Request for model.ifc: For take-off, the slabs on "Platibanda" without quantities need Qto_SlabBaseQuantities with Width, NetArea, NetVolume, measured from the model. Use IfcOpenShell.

First a look at what the model holds.

```python
import ifcopenshell
import ifcopenshell.util.element
import ifcopenshell.util.unit

model = ifcopenshell.open("model.ifc")
print(model.schema)
for unit_type in ("LENGTHUNIT", "AREAUNIT", "VOLUMEUNIT"):
    print(unit_type, ifcopenshell.util.unit.calculate_unit_scale(model, unit_type))
storey = next(s for s in model.by_type("IfcBuildingStorey") if s.Name == "Platibanda")
slabs = [e for e in ifcopenshell.util.element.get_decomposition(storey) if e.is_a("IfcSlab")]
for e in sorted(slabs, key=lambda e: e.id()):
    print(e.id(), e.is_a(), e.Name, list(ifcopenshell.util.element.get_psets(e, qtos_only=True)), sep=" | ")
```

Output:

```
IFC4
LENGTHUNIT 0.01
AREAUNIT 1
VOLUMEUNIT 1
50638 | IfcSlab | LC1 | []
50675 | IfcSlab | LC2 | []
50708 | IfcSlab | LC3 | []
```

```python
import ifcopenshell
import ifcopenshell.api.pset
import ifcopenshell.geom
import ifcopenshell.util.element
import ifcopenshell.util.shape
import ifcopenshell.util.unit

model = ifcopenshell.open("model.ifc")
unit_scale = ifcopenshell.util.unit.calculate_unit_scale(model)
area_scale = ifcopenshell.util.unit.calculate_unit_scale(model, "AREAUNIT")
volume_scale = ifcopenshell.util.unit.calculate_unit_scale(model, "VOLUMEUNIT")
settings = ifcopenshell.geom.settings()

storey = next(s for s in model.by_type("IfcBuildingStorey") if s.Name == "Platibanda")
slabs = [e for e in ifcopenshell.util.element.get_decomposition(storey) if e.is_a("IfcSlab")]

for e in sorted(slabs, key=lambda e: e.id()):
    if ifcopenshell.util.element.get_psets(e, qtos_only=True, should_inherit=False):
        continue
    # Geometry comes back in metres, in the element's own axes.
    shape = ifcopenshell.geom.create_shape(settings, e)
    values = {
        "Width": ifcopenshell.util.shape.get_z(shape.geometry) / unit_scale,
        "NetArea": ifcopenshell.util.shape.get_footprint_area(shape.geometry) / area_scale,
        "NetVolume": ifcopenshell.util.shape.get_volume(shape.geometry) / volume_scale,
    }
    qto = ifcopenshell.api.pset.add_qto(model, product=e, name="Qto_SlabBaseQuantities")
    ifcopenshell.api.pset.edit_qto(model, qto=qto, properties=values)
    print(e.id(), {k: round(v, 3) for k, v in values.items()})

model.write("model_rev.ifc")
```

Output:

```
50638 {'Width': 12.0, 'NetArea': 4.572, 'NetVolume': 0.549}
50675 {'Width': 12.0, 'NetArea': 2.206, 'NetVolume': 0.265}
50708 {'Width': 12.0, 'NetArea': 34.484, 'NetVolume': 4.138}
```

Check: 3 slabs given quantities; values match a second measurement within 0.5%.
